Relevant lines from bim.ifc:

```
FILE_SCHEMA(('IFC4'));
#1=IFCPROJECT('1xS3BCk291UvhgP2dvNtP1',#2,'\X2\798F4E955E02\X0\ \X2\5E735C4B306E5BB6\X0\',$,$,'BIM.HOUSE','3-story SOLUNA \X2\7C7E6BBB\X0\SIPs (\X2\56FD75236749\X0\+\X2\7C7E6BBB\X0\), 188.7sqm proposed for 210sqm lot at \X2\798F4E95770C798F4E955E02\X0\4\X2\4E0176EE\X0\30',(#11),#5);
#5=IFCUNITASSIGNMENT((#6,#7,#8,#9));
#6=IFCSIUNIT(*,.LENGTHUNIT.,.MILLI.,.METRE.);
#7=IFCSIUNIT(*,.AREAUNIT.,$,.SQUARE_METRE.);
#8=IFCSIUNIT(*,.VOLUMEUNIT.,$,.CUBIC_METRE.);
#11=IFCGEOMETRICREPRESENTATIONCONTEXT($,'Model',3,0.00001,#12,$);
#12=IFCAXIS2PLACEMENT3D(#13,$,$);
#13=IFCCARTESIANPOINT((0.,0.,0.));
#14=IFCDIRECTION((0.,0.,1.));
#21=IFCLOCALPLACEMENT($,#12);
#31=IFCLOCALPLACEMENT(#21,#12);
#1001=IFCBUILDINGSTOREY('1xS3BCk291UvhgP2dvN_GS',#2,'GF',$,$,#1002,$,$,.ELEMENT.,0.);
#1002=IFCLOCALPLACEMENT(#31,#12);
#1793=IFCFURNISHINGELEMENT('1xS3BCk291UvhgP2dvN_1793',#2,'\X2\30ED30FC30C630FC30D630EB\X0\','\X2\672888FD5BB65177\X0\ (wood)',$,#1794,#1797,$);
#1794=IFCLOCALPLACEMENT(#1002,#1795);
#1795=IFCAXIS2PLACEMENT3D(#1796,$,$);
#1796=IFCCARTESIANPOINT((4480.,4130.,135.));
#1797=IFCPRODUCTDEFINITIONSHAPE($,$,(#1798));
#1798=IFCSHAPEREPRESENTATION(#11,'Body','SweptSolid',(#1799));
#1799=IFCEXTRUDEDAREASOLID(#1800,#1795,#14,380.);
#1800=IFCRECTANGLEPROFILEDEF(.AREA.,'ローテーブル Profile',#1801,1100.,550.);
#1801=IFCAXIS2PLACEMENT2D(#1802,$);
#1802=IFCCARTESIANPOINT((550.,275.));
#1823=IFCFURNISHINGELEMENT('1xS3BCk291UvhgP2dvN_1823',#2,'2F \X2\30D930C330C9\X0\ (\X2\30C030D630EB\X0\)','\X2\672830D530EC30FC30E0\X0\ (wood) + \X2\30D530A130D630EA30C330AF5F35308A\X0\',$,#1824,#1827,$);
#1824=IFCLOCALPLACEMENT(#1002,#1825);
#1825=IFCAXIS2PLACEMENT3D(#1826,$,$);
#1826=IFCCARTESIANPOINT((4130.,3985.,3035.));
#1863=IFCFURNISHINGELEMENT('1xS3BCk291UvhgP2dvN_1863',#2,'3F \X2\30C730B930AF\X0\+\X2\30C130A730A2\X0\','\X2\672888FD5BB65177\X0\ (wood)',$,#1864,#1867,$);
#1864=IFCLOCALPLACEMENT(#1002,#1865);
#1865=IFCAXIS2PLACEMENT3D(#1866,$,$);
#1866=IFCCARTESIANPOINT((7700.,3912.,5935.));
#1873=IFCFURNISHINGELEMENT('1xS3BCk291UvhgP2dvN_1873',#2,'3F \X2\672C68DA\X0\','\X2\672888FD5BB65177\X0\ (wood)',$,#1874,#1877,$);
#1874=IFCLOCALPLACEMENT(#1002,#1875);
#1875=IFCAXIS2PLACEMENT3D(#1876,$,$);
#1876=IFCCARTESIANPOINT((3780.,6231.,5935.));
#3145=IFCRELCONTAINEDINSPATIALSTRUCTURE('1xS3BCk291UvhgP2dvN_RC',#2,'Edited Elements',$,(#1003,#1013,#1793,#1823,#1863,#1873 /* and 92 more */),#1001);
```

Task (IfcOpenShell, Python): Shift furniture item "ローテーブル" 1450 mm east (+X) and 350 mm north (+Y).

```python
import ifcopenshell
import ifcopenshell.api.geometry
import ifcopenshell.util.placement
import ifcopenshell.util.unit

model = ifcopenshell.open("bim.ifc")
unit_scale = ifcopenshell.util.unit.calculate_unit_scale(model)

item = model.by_id(1793)
matrix = ifcopenshell.util.placement.get_local_placement(item.ObjectPlacement)
matrix[0, 3] += 1.45 / unit_scale
matrix[1, 3] += 0.35 / unit_scale
ifcopenshell.api.geometry.edit_object_placement(model, product=item, matrix=matrix, is_si=False)

print(ifcopenshell.util.placement.get_local_placement(item.ObjectPlacement).round(3) + 0.0)

model.write("bim-out.ifc")
```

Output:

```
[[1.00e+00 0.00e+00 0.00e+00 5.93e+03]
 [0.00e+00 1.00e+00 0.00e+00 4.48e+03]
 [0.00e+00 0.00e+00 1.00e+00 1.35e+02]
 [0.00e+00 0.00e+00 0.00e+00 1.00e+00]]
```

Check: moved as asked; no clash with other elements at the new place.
